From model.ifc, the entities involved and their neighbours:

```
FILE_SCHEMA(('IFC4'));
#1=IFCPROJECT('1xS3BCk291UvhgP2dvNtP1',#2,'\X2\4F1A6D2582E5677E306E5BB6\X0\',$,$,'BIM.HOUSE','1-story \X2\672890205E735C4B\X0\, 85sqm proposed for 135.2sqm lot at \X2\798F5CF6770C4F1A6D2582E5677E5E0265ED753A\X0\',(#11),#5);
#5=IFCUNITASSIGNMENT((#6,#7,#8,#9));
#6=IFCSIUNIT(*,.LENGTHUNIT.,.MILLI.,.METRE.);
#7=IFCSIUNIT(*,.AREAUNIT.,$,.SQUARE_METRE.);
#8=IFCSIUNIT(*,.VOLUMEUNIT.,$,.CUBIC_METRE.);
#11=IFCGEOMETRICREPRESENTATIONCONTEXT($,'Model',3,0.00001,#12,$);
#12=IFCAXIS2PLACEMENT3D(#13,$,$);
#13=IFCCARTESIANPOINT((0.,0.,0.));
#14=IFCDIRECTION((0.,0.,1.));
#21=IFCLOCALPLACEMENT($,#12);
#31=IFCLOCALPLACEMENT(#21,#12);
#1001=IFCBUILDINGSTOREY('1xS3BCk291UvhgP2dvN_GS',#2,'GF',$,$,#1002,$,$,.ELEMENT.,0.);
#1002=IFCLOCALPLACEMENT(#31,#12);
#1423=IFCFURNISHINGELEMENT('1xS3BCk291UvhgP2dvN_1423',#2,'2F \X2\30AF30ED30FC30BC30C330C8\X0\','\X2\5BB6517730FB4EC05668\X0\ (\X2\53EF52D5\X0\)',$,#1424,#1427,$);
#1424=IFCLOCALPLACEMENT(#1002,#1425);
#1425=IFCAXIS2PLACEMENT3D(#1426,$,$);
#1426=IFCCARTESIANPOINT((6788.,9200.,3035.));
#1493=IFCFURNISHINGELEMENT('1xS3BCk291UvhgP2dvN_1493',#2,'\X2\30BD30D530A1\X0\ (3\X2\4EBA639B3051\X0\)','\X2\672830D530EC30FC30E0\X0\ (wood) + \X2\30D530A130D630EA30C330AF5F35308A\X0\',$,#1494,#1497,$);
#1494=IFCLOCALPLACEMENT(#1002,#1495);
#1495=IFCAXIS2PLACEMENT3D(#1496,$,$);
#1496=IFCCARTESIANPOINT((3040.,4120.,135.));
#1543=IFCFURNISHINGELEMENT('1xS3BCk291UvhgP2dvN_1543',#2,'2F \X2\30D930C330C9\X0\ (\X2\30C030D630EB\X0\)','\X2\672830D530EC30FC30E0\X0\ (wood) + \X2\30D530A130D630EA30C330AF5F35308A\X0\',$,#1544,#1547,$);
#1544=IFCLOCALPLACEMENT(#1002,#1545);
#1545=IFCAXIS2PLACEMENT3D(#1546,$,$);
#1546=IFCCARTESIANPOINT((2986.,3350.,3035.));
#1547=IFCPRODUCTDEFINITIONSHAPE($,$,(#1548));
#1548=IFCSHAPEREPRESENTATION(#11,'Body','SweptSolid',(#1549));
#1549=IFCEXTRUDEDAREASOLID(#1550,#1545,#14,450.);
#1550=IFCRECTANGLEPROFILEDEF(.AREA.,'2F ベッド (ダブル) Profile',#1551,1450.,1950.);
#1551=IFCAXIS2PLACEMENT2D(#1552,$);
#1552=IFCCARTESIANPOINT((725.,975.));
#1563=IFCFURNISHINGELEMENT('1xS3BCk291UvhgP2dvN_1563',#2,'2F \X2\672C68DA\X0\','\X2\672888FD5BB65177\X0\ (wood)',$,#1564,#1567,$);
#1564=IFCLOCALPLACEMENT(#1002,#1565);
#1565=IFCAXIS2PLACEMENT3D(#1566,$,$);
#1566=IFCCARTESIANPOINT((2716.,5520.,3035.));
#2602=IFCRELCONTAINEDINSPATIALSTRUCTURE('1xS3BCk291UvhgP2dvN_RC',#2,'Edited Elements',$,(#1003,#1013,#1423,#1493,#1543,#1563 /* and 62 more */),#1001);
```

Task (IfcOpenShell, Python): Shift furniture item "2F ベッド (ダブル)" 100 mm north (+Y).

```python
import ifcopenshell
import ifcopenshell.api.geometry
import ifcopenshell.util.placement
import ifcopenshell.util.unit

model = ifcopenshell.open("model.ifc")
unit_scale = ifcopenshell.util.unit.calculate_unit_scale(model)

item = model.by_guid("1xS3BCk291UvhgP2dvN_1543")
matrix = ifcopenshell.util.placement.get_local_placement(item.ObjectPlacement)
matrix[1, 3] += 0.1 / unit_scale
ifcopenshell.api.geometry.edit_object_placement(model, product=item, matrix=matrix, is_si=False)

print(ifcopenshell.util.placement.get_local_placement(item.ObjectPlacement).round(3) + 0.0)

model.write("model_v2.ifc")
```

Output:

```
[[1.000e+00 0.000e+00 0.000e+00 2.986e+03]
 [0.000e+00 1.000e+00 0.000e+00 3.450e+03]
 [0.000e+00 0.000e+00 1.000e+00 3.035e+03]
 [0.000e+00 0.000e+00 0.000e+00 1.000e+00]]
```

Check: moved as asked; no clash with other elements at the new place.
